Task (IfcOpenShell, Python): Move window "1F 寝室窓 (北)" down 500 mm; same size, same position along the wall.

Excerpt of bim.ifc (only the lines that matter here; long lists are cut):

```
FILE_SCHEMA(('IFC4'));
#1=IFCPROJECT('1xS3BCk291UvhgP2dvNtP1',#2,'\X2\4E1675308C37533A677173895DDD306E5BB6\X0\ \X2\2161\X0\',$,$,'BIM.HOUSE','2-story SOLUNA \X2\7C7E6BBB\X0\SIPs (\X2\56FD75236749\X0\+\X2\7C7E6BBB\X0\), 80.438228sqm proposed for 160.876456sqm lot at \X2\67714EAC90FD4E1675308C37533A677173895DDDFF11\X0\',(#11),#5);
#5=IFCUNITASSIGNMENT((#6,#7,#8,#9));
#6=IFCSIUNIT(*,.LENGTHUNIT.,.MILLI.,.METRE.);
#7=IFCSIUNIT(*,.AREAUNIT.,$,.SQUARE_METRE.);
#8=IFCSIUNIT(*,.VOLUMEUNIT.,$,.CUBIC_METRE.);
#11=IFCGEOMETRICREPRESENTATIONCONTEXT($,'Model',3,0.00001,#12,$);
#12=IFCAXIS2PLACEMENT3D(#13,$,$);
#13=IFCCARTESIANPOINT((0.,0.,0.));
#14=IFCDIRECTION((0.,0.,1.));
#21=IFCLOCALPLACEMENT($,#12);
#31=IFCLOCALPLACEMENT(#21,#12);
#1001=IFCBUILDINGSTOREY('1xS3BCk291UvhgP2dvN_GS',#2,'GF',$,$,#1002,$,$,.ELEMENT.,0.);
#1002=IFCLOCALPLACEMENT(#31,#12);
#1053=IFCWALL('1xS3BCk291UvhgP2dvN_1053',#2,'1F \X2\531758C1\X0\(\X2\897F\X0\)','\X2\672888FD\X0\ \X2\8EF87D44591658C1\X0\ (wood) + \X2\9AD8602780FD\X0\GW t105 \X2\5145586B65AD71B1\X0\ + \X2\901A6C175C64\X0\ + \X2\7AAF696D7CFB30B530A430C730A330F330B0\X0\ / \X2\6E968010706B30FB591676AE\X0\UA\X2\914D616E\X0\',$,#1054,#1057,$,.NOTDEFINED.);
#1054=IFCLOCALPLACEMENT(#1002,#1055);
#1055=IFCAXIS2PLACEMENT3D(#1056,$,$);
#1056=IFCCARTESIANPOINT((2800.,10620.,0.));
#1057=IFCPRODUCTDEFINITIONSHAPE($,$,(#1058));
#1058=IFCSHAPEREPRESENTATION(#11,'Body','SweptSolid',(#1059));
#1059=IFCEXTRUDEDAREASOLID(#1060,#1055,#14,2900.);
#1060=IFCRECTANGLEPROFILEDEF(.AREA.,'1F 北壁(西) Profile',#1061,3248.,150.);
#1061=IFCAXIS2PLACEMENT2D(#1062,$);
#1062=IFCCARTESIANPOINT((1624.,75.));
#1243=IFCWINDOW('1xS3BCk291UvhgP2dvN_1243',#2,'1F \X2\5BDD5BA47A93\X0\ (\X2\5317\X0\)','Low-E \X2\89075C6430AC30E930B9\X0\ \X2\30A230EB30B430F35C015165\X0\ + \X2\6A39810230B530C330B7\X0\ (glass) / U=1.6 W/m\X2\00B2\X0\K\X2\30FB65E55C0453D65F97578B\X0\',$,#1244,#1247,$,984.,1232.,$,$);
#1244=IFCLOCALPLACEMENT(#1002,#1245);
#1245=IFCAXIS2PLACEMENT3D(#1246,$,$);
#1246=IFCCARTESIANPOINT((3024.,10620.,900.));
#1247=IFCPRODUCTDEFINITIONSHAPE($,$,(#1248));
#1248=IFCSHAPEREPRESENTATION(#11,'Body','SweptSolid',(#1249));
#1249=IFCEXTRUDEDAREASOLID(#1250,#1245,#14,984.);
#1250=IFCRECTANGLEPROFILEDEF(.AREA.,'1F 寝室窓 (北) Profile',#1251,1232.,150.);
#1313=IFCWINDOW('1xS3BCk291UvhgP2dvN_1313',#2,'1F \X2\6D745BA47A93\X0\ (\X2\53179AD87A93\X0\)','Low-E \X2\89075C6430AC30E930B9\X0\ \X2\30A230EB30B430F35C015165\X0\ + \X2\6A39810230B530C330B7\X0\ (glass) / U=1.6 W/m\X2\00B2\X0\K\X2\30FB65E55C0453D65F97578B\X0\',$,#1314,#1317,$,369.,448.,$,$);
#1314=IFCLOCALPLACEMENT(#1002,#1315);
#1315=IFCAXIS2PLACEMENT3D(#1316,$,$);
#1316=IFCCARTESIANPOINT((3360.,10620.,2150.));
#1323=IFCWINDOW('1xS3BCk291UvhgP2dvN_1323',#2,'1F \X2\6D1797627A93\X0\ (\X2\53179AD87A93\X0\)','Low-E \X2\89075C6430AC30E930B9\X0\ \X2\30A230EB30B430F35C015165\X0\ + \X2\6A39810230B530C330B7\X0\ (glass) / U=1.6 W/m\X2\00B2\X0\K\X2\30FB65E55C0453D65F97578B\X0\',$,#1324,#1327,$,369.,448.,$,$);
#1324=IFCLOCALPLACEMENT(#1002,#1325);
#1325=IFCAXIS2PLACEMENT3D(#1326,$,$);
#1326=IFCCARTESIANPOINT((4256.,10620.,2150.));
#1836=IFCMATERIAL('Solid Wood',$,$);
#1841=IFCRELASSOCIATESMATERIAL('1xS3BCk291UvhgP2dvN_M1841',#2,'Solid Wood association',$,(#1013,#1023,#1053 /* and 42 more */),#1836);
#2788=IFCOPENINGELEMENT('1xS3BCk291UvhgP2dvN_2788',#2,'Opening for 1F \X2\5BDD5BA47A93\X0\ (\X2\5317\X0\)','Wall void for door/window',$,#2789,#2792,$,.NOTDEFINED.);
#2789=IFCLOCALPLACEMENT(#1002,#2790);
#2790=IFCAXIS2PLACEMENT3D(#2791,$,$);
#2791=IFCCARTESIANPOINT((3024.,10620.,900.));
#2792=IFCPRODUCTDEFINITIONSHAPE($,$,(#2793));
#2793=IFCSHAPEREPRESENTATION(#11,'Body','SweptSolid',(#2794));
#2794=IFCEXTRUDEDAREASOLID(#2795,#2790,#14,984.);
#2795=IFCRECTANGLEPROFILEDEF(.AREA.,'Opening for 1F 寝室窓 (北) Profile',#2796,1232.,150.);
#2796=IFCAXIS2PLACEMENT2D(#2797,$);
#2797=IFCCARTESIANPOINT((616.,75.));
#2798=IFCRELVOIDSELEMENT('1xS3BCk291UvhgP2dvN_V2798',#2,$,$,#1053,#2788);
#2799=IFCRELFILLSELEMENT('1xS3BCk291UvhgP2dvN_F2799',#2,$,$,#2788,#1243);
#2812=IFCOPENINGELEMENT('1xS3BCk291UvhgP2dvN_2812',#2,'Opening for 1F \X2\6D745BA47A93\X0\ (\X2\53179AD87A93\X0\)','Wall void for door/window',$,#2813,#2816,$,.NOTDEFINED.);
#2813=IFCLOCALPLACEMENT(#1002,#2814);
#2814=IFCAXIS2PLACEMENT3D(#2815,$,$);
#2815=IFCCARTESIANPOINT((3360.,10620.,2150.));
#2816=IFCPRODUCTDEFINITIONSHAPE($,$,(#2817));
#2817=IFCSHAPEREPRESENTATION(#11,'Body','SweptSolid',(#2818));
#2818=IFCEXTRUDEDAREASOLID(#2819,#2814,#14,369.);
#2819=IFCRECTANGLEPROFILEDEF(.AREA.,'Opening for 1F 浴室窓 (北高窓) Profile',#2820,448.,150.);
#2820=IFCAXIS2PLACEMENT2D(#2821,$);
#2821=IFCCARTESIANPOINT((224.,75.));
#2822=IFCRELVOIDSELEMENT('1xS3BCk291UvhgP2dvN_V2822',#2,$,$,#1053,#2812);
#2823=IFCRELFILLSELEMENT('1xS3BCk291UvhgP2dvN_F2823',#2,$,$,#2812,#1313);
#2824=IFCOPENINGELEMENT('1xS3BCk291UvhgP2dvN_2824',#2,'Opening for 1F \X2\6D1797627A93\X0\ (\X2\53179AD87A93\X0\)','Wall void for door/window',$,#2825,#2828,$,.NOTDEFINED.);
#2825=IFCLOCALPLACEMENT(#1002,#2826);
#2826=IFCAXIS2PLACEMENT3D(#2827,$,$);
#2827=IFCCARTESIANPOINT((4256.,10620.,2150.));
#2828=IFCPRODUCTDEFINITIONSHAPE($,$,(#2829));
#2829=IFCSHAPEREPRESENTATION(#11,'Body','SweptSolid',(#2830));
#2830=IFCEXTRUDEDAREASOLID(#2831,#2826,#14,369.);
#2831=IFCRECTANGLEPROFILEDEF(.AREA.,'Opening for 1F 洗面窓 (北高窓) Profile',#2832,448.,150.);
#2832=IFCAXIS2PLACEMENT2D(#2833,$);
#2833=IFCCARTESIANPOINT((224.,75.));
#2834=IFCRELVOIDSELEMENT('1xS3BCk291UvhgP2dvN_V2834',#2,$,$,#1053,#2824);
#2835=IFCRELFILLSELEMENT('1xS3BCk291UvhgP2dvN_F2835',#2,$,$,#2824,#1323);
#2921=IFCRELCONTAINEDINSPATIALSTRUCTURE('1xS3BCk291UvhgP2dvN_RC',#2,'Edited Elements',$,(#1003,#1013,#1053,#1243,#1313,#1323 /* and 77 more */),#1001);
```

```python
import numpy as np
import ifcopenshell
import ifcopenshell.api.geometry
import ifcopenshell.util.placement
import ifcopenshell.util.unit

model = ifcopenshell.open("bim.ifc")
unit_scale = ifcopenshell.util.unit.calculate_unit_scale(model)

window = model.by_guid("1xS3BCk291UvhgP2dvN_1243")
opening = window.FillsVoids[0].RelatingOpeningElement
dz = -500.0

shift = np.array([0.0, 0.0, dz])
# The window is not placed relative to its opening, so move both.
for product in (opening, window):
    matrix = ifcopenshell.util.placement.get_local_placement(product.ObjectPlacement)
    matrix[:3, 3] += shift
    ifcopenshell.api.geometry.edit_object_placement(model, product=product, matrix=matrix, is_si=False)

print(f"moved by {dz * unit_scale:+.3f} m")

model.write("bim_rev.ifc")
```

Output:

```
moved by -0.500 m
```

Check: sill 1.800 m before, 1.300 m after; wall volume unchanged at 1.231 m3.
